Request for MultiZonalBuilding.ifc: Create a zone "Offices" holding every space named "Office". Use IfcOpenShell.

First a look at what the model holds.

```python
import ifcopenshell

model = ifcopenshell.open("MultiZonalBuilding.ifc")
print(model.schema)
seen = {}
for space in model.by_type("IfcSpace"):
    seen[space.LongName] = seen.get(space.LongName, 0) + 1
for name, count in sorted(seen.items(), key=str):
    print(count, "x", name)
print("zones:", [z.Name for z in model.by_type("IfcZone")][:20])
```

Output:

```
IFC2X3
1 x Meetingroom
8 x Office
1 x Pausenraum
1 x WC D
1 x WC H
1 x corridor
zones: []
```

```python
import ifcopenshell
import ifcopenshell.api.group
import ifcopenshell.api.root

model = ifcopenshell.open("MultiZonalBuilding.ifc")

names = {"Office"}
spaces = [s for s in model.by_type("IfcSpace") if s.LongName in names]

zone = ifcopenshell.api.root.create_entity(model, ifc_class="IfcZone", name="Offices")
ifcopenshell.api.group.assign_group(model, products=spaces, group=zone)
print(len(spaces), "spaces in", zone.Name)

model.write("MultiZonalBuilding_v2.ifc")
```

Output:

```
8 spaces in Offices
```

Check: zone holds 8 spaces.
